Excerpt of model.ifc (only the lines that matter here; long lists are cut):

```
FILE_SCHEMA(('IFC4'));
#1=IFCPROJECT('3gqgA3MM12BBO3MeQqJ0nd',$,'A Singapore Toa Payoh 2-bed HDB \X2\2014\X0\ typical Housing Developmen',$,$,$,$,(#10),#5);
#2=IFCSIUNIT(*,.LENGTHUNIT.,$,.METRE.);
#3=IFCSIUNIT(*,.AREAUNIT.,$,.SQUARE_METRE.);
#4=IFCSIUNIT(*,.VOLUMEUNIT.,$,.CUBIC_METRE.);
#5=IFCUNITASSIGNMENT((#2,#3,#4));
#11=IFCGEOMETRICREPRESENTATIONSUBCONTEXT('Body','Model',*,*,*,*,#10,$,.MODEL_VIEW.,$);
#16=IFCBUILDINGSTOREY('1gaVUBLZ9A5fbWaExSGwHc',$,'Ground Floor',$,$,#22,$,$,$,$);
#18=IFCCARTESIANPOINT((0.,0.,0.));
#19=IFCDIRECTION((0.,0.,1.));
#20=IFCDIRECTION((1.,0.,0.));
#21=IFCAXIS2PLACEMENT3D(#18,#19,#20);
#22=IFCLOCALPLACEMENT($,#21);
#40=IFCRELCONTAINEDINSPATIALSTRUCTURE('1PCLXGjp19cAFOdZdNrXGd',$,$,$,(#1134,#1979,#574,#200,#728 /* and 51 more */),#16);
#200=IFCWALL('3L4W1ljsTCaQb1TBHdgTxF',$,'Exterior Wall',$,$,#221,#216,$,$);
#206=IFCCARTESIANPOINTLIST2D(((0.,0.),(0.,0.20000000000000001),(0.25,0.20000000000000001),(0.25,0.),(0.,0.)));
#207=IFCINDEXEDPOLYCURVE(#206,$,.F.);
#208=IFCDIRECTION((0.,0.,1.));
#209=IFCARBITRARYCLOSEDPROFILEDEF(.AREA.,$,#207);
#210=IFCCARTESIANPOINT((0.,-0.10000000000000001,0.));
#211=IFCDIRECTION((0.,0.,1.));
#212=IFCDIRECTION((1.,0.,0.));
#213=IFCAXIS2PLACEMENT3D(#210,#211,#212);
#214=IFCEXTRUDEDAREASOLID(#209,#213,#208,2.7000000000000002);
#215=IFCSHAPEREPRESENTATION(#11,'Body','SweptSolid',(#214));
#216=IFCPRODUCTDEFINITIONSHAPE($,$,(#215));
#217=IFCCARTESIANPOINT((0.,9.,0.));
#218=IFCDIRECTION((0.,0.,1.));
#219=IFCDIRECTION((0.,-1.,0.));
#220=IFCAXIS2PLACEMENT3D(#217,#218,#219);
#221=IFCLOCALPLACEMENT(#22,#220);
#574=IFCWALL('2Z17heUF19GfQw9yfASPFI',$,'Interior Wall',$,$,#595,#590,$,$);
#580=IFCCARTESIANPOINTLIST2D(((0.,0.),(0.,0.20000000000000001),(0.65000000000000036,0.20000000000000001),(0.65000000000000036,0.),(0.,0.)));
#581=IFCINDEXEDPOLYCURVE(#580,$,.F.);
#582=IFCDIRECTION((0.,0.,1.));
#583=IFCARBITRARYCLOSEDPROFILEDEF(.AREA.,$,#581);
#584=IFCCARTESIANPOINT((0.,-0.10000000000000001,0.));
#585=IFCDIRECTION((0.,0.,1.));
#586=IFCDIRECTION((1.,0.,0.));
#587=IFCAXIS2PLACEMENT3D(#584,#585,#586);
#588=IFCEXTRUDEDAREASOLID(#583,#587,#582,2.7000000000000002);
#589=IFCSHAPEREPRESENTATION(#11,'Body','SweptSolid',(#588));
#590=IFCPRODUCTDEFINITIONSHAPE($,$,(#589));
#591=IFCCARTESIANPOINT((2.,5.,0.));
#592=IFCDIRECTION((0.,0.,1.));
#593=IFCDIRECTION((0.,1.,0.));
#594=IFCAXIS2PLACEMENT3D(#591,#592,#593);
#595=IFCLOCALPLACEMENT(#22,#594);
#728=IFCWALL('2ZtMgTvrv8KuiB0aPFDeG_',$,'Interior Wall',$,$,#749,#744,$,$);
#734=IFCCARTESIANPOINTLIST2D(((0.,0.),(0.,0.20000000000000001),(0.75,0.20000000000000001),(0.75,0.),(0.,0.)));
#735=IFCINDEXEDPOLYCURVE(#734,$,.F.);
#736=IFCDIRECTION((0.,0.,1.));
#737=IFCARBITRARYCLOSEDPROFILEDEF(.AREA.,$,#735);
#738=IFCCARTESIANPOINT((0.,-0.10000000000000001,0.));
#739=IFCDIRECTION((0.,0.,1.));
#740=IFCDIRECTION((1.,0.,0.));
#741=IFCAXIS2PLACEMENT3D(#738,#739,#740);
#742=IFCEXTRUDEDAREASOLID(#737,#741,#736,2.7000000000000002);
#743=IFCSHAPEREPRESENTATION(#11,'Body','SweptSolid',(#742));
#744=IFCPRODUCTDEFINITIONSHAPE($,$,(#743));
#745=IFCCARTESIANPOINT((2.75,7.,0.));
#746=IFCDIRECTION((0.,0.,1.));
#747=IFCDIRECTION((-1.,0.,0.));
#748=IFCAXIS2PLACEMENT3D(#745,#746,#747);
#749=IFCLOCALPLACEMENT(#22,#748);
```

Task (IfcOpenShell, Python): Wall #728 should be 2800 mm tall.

```python
import ifcopenshell
import ifcopenshell.geom
import ifcopenshell.util.representation
import ifcopenshell.util.shape
import ifcopenshell.util.unit

model = ifcopenshell.open("model.ifc")
unit_scale = ifcopenshell.util.unit.calculate_unit_scale(model)
settings = ifcopenshell.geom.settings()


def volume(element):
    """Net volume in cubic metres, openings subtracted."""
    shape = ifcopenshell.geom.create_shape(settings, element)
    return ifcopenshell.util.shape.get_volume(shape.geometry)


wall = model.by_guid("2ZtMgTvrv8KuiB0aPFDeG_")
before = volume(wall)

body = ifcopenshell.util.representation.get_representation(wall, "Model", "Body")
solid = body.Items[0]
old_height = solid.Depth
solid.Depth = 2.8 / unit_scale
after = volume(wall)

print(f"height {old_height:g} -> {solid.Depth:g}, volume {before:.3f} -> {after:.3f} m3")

model.write("model-out.ifc")
```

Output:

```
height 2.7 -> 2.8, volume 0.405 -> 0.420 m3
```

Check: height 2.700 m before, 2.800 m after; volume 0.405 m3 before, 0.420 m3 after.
